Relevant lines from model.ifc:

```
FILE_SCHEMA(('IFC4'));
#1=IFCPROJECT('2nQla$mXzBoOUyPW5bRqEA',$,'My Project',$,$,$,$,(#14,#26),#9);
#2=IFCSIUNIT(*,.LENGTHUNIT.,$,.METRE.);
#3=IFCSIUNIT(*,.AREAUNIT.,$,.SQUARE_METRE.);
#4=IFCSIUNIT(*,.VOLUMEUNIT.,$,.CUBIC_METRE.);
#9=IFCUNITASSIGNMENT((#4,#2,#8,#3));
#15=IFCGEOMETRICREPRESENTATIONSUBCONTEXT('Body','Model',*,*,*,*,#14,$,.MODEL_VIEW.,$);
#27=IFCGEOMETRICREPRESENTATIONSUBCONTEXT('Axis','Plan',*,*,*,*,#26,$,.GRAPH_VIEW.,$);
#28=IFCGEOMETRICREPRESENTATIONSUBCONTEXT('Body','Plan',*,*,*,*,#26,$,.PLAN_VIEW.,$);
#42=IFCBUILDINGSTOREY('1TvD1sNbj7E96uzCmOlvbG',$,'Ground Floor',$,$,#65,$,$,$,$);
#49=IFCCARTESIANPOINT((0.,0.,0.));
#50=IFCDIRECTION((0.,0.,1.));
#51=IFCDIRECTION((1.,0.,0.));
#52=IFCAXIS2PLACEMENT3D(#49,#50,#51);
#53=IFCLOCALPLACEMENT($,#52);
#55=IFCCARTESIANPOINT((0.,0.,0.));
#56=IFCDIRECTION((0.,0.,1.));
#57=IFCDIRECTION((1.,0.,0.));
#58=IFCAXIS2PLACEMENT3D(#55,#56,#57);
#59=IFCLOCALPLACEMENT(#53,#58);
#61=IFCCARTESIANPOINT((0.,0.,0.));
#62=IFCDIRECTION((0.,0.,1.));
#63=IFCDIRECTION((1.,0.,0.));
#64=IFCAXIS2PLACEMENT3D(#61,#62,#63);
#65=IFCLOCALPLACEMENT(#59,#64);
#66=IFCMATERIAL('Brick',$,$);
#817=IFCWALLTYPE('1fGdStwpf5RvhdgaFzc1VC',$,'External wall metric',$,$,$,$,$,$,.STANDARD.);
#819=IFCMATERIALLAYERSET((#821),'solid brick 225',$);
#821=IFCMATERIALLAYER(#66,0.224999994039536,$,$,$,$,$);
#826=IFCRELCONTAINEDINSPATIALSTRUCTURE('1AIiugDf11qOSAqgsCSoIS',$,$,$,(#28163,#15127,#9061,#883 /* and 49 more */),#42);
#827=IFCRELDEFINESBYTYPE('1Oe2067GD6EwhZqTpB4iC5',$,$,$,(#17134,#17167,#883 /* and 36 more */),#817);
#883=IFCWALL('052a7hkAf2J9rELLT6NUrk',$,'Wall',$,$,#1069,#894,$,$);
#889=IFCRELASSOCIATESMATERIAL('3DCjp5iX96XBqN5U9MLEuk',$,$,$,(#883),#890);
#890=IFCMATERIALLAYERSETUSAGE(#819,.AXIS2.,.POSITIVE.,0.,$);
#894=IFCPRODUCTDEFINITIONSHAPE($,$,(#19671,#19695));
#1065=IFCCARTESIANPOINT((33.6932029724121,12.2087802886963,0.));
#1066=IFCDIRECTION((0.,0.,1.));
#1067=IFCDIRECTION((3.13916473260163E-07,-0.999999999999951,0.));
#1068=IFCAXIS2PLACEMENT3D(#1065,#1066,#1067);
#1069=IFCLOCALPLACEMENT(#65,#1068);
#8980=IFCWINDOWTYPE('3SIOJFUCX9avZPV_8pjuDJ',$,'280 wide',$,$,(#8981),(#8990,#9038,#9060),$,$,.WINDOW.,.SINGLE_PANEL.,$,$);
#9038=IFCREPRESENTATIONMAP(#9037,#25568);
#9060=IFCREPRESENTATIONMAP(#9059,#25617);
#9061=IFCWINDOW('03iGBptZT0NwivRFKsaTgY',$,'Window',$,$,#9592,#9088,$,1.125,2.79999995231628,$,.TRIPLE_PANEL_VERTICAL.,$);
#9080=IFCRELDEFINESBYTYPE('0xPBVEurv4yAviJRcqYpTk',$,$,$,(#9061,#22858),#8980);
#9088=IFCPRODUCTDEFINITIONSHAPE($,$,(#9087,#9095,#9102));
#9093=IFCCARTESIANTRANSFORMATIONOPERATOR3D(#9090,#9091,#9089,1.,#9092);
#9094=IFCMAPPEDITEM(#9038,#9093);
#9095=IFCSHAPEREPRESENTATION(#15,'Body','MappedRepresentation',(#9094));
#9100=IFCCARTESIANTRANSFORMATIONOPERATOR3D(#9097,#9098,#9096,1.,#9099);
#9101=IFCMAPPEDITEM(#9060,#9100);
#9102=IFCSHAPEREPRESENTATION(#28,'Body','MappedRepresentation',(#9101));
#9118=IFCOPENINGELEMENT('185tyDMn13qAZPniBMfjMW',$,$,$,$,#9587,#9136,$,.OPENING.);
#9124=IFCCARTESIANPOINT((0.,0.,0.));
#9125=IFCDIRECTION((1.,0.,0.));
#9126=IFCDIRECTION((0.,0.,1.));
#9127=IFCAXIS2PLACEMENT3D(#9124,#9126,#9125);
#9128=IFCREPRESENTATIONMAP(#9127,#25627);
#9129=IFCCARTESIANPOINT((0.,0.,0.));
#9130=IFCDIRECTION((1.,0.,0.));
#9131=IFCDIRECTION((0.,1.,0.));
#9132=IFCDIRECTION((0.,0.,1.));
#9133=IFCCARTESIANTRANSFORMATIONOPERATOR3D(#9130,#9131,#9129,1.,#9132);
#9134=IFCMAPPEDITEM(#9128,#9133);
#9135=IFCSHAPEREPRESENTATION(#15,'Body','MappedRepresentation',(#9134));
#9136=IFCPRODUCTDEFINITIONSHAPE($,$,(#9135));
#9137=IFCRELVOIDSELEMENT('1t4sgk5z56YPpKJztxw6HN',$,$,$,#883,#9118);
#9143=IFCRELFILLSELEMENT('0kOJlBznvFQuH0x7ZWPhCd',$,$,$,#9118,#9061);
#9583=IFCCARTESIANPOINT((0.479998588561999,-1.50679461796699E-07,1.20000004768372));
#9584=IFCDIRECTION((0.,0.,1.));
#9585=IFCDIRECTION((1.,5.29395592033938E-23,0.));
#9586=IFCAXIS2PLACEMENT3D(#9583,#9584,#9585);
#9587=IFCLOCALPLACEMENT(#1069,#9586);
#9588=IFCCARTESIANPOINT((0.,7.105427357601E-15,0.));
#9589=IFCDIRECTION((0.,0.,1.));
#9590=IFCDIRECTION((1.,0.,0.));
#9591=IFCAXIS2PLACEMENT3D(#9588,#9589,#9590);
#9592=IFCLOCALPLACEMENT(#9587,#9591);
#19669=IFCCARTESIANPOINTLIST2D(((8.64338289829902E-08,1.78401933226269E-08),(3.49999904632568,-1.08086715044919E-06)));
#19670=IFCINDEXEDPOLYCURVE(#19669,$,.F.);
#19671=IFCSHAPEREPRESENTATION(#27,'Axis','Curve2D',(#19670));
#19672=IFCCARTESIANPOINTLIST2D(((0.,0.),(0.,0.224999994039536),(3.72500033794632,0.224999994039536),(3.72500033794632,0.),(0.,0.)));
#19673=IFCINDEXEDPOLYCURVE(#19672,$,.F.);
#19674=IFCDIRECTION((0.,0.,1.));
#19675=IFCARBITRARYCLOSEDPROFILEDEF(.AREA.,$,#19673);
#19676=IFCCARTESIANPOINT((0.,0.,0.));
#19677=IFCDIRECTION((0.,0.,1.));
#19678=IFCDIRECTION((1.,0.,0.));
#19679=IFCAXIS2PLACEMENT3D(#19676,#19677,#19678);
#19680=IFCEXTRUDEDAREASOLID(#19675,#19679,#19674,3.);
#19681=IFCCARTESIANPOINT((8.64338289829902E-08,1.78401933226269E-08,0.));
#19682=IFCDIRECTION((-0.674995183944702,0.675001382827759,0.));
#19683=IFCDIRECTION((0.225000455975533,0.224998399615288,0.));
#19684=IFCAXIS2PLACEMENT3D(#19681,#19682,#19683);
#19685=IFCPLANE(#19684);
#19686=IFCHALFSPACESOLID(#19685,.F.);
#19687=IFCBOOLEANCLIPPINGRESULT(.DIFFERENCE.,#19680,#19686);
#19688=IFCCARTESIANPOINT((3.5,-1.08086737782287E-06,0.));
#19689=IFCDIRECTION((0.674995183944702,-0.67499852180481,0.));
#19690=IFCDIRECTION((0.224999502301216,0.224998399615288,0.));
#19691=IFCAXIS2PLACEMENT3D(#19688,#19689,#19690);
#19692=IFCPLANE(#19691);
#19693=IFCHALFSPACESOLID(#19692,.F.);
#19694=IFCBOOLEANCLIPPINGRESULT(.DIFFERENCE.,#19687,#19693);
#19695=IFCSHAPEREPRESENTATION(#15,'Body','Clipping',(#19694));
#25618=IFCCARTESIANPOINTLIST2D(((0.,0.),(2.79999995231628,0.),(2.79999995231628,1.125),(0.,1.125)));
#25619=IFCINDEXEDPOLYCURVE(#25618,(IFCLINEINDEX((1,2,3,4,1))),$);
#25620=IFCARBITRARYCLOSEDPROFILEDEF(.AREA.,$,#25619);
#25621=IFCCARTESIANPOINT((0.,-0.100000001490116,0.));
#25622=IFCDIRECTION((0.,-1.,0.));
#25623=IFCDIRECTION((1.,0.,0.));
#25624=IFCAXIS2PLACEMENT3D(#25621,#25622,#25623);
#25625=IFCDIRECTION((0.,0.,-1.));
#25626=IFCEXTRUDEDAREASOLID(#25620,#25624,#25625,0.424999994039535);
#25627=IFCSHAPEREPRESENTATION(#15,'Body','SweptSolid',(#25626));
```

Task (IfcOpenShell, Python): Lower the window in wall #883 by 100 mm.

```python
import numpy as np
import ifcopenshell
import ifcopenshell.api.geometry
import ifcopenshell.util.placement
import ifcopenshell.util.unit

model = ifcopenshell.open("model.ifc")
unit_scale = ifcopenshell.util.unit.calculate_unit_scale(model)

window = model.by_id(9061)
opening = window.FillsVoids[0].RelatingOpeningElement
dz = -0.1

shift = np.array([0.0, 0.0, dz])
# The window is placed relative to its opening, so it follows when the opening moves.
matrix = ifcopenshell.util.placement.get_local_placement(opening.ObjectPlacement)
matrix[:3, 3] += shift
ifcopenshell.api.geometry.edit_object_placement(
    model, product=opening, matrix=matrix, is_si=False, should_transform_children=True
)

print(f"moved by {dz * unit_scale:+.3f} m")

model.write("model_updated.ifc")
```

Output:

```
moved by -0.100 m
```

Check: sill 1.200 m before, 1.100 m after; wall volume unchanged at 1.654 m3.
